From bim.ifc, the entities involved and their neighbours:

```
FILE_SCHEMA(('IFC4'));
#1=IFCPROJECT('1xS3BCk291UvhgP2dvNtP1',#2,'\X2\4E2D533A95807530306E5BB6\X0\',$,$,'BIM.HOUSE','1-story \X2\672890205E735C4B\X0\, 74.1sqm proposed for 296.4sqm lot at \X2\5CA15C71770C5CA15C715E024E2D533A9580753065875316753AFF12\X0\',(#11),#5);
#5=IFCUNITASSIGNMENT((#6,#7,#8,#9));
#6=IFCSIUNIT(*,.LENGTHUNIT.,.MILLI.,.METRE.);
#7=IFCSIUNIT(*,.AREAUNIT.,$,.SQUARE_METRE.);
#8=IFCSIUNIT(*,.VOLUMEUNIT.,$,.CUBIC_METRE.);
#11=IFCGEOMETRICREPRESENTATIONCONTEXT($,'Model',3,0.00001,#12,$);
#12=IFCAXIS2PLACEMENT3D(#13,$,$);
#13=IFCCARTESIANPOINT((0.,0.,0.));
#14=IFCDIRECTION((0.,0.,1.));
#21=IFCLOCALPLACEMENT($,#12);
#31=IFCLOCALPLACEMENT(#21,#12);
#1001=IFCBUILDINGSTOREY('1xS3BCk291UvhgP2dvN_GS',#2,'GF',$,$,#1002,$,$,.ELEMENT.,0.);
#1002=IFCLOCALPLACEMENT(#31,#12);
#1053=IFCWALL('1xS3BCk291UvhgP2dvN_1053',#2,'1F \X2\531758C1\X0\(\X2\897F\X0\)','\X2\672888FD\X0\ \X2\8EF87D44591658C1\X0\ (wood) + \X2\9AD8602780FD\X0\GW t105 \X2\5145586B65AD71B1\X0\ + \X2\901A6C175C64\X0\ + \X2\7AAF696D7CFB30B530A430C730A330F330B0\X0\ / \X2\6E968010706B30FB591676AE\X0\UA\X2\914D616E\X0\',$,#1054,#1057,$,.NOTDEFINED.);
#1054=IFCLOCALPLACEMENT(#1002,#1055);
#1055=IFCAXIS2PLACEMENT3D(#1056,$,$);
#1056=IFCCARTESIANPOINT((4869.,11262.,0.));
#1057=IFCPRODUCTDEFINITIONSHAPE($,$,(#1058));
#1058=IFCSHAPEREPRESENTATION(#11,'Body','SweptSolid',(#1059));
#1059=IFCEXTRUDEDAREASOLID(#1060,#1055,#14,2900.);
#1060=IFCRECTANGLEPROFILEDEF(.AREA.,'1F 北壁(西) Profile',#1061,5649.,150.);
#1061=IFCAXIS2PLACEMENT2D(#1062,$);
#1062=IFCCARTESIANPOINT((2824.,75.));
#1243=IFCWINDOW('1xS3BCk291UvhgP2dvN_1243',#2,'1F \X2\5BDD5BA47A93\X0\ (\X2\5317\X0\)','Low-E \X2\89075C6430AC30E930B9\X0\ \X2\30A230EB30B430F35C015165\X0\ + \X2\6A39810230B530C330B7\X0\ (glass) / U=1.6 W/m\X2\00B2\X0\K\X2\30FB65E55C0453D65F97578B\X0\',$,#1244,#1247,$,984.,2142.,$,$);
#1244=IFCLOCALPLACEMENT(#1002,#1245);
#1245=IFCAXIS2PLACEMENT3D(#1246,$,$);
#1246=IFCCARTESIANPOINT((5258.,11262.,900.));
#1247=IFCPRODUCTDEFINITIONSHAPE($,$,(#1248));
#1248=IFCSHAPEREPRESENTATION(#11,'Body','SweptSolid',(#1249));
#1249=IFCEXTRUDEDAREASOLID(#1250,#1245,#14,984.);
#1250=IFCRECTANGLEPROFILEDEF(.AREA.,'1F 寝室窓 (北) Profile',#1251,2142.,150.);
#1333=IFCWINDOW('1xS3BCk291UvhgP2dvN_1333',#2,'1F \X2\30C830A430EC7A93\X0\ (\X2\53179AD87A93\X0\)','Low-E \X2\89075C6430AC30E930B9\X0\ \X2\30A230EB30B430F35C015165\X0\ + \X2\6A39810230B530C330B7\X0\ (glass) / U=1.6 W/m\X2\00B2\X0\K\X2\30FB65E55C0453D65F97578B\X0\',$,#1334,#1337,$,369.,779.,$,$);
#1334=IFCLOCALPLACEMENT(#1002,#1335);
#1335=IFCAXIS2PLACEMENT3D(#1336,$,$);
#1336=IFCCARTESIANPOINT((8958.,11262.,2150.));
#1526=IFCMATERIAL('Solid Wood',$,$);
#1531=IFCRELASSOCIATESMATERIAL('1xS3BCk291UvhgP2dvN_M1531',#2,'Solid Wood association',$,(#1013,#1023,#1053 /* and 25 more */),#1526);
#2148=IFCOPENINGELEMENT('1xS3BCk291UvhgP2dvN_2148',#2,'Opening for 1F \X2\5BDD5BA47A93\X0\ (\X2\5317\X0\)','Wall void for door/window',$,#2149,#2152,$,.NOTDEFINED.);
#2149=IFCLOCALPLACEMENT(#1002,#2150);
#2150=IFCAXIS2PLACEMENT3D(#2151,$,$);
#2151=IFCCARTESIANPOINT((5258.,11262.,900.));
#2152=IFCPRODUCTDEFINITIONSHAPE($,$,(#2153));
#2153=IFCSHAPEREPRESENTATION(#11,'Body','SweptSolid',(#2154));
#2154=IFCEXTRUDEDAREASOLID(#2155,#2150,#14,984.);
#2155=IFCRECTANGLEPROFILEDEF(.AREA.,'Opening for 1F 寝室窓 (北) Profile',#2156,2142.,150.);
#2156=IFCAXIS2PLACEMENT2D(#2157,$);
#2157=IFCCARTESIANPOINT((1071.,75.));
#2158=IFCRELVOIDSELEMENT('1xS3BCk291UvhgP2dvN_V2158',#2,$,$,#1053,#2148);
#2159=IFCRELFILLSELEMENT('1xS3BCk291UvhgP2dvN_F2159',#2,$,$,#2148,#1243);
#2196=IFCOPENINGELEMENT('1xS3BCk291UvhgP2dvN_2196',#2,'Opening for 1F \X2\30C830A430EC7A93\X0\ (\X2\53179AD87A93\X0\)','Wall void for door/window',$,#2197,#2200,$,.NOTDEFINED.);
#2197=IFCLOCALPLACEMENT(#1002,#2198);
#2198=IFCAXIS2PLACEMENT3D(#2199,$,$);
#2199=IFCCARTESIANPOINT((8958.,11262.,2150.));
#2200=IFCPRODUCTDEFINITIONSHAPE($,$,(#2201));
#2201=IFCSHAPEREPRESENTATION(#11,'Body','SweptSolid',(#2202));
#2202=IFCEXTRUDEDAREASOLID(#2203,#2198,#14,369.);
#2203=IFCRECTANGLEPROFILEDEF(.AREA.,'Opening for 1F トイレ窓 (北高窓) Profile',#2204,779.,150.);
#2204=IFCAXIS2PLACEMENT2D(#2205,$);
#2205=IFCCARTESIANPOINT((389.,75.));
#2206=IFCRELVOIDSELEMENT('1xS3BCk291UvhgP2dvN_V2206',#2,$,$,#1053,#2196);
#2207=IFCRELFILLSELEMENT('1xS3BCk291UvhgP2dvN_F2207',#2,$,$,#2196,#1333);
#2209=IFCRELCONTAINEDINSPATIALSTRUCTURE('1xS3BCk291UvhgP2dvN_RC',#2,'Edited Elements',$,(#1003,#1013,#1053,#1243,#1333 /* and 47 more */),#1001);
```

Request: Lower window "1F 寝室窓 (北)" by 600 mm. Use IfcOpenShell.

```python
import numpy as np
import ifcopenshell
import ifcopenshell.api.geometry
import ifcopenshell.util.placement
import ifcopenshell.util.unit

model = ifcopenshell.open("bim.ifc")
unit_scale = ifcopenshell.util.unit.calculate_unit_scale(model)

window = model.by_guid("1xS3BCk291UvhgP2dvN_1243")
opening = window.FillsVoids[0].RelatingOpeningElement
dz = -600.0

shift = np.array([0.0, 0.0, dz])
# The window is not placed relative to its opening, so move both.
for product in (opening, window):
    matrix = ifcopenshell.util.placement.get_local_placement(product.ObjectPlacement)
    matrix[:3, 3] += shift
    ifcopenshell.api.geometry.edit_object_placement(model, product=product, matrix=matrix, is_si=False)

print(f"moved by {dz * unit_scale:+.3f} m")

model.write("bim_v2.ifc")
```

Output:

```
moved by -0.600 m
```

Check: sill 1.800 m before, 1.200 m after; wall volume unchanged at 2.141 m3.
